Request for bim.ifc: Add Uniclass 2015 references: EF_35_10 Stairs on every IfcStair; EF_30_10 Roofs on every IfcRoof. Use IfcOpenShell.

First a look at what the model holds.

```python
import ifcopenshell

model = ifcopenshell.open("bim.ifc")
print(model.schema)
print("classifications:", [c.Name for c in model.by_type("IfcClassification")])
for ifc_class in ("IfcDoor", "IfcRoof", "IfcStair", "IfcWall", "IfcWindow"):
    print(ifc_class, len(model.by_type(ifc_class)))
```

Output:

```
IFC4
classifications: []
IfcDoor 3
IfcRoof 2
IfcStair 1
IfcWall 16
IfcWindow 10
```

```python
import ifcopenshell
import ifcopenshell.api.classification

model = ifcopenshell.open("bim.ifc")

system = ifcopenshell.api.classification.add_classification(model, classification="Uniclass 2015")

codes = {
    "IfcStair": ("EF_35_10", "Stairs"),
    "IfcRoof": ("EF_30_10", "Roofs"),
}
for ifc_class, (code, name) in codes.items():
    products = model.by_type(ifc_class)
    ifcopenshell.api.classification.add_reference(
        model, products=products, classification=system, identification=code, name=name
    )
    print(code, len(products))

model.write("bim-out.ifc")
```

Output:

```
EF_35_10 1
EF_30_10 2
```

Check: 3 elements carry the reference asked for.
